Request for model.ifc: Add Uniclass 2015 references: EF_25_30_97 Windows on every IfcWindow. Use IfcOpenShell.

First a look at what the model holds.

```python
import ifcopenshell

model = ifcopenshell.open("model.ifc")
print(model.schema)
print("classifications:", [c.Name for c in model.by_type("IfcClassification")])
for ifc_class in ("IfcDoor", "IfcRoof", "IfcStair", "IfcWall", "IfcWindow"):
    print(ifc_class, len(model.by_type(ifc_class)))
```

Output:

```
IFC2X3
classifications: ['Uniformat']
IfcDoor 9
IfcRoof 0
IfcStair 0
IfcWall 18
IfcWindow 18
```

```python
import ifcopenshell
import ifcopenshell.api.classification

model = ifcopenshell.open("model.ifc")

# IFC2X3 requires Source and Edition and has no link from the project to the system.
system = model.create_entity("IfcClassification", Source="NBS", Edition="2015", Name="Uniclass 2015")

codes = {
    "IfcWindow": ("EF_25_30_97", "Windows"),
}
for ifc_class, (code, name) in codes.items():
    products = model.by_type(ifc_class)
    ifcopenshell.api.classification.add_reference(
        model, products=products, classification=system, identification=code, name=name
    )
    print(code, len(products))

model.write("model_updated.ifc")
```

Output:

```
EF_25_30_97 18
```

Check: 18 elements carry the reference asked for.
